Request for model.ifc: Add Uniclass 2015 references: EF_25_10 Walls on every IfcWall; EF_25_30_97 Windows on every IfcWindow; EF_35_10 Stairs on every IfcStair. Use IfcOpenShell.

First a look at what the model holds.

```python
import ifcopenshell

model = ifcopenshell.open("model.ifc")
print(model.schema)
print("classifications:", [c.Name for c in model.by_type("IfcClassification")])
for ifc_class in ("IfcDoor", "IfcRoof", "IfcStair", "IfcWall", "IfcWindow"):
    print(ifc_class, len(model.by_type(ifc_class)))
```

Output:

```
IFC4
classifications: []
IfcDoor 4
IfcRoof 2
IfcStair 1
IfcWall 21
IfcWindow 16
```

```python
import ifcopenshell
import ifcopenshell.api.classification

model = ifcopenshell.open("model.ifc")

system = ifcopenshell.api.classification.add_classification(model, classification="Uniclass 2015")

codes = {
    "IfcWall": ("EF_25_10", "Walls"),
    "IfcWindow": ("EF_25_30_97", "Windows"),
    "IfcStair": ("EF_35_10", "Stairs"),
}
for ifc_class, (code, name) in codes.items():
    products = model.by_type(ifc_class)
    ifcopenshell.api.classification.add_reference(
        model, products=products, classification=system, identification=code, name=name
    )
    print(code, len(products))

model.write("model_v2.ifc")
```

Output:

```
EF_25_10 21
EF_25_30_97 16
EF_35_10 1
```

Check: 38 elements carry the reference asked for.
